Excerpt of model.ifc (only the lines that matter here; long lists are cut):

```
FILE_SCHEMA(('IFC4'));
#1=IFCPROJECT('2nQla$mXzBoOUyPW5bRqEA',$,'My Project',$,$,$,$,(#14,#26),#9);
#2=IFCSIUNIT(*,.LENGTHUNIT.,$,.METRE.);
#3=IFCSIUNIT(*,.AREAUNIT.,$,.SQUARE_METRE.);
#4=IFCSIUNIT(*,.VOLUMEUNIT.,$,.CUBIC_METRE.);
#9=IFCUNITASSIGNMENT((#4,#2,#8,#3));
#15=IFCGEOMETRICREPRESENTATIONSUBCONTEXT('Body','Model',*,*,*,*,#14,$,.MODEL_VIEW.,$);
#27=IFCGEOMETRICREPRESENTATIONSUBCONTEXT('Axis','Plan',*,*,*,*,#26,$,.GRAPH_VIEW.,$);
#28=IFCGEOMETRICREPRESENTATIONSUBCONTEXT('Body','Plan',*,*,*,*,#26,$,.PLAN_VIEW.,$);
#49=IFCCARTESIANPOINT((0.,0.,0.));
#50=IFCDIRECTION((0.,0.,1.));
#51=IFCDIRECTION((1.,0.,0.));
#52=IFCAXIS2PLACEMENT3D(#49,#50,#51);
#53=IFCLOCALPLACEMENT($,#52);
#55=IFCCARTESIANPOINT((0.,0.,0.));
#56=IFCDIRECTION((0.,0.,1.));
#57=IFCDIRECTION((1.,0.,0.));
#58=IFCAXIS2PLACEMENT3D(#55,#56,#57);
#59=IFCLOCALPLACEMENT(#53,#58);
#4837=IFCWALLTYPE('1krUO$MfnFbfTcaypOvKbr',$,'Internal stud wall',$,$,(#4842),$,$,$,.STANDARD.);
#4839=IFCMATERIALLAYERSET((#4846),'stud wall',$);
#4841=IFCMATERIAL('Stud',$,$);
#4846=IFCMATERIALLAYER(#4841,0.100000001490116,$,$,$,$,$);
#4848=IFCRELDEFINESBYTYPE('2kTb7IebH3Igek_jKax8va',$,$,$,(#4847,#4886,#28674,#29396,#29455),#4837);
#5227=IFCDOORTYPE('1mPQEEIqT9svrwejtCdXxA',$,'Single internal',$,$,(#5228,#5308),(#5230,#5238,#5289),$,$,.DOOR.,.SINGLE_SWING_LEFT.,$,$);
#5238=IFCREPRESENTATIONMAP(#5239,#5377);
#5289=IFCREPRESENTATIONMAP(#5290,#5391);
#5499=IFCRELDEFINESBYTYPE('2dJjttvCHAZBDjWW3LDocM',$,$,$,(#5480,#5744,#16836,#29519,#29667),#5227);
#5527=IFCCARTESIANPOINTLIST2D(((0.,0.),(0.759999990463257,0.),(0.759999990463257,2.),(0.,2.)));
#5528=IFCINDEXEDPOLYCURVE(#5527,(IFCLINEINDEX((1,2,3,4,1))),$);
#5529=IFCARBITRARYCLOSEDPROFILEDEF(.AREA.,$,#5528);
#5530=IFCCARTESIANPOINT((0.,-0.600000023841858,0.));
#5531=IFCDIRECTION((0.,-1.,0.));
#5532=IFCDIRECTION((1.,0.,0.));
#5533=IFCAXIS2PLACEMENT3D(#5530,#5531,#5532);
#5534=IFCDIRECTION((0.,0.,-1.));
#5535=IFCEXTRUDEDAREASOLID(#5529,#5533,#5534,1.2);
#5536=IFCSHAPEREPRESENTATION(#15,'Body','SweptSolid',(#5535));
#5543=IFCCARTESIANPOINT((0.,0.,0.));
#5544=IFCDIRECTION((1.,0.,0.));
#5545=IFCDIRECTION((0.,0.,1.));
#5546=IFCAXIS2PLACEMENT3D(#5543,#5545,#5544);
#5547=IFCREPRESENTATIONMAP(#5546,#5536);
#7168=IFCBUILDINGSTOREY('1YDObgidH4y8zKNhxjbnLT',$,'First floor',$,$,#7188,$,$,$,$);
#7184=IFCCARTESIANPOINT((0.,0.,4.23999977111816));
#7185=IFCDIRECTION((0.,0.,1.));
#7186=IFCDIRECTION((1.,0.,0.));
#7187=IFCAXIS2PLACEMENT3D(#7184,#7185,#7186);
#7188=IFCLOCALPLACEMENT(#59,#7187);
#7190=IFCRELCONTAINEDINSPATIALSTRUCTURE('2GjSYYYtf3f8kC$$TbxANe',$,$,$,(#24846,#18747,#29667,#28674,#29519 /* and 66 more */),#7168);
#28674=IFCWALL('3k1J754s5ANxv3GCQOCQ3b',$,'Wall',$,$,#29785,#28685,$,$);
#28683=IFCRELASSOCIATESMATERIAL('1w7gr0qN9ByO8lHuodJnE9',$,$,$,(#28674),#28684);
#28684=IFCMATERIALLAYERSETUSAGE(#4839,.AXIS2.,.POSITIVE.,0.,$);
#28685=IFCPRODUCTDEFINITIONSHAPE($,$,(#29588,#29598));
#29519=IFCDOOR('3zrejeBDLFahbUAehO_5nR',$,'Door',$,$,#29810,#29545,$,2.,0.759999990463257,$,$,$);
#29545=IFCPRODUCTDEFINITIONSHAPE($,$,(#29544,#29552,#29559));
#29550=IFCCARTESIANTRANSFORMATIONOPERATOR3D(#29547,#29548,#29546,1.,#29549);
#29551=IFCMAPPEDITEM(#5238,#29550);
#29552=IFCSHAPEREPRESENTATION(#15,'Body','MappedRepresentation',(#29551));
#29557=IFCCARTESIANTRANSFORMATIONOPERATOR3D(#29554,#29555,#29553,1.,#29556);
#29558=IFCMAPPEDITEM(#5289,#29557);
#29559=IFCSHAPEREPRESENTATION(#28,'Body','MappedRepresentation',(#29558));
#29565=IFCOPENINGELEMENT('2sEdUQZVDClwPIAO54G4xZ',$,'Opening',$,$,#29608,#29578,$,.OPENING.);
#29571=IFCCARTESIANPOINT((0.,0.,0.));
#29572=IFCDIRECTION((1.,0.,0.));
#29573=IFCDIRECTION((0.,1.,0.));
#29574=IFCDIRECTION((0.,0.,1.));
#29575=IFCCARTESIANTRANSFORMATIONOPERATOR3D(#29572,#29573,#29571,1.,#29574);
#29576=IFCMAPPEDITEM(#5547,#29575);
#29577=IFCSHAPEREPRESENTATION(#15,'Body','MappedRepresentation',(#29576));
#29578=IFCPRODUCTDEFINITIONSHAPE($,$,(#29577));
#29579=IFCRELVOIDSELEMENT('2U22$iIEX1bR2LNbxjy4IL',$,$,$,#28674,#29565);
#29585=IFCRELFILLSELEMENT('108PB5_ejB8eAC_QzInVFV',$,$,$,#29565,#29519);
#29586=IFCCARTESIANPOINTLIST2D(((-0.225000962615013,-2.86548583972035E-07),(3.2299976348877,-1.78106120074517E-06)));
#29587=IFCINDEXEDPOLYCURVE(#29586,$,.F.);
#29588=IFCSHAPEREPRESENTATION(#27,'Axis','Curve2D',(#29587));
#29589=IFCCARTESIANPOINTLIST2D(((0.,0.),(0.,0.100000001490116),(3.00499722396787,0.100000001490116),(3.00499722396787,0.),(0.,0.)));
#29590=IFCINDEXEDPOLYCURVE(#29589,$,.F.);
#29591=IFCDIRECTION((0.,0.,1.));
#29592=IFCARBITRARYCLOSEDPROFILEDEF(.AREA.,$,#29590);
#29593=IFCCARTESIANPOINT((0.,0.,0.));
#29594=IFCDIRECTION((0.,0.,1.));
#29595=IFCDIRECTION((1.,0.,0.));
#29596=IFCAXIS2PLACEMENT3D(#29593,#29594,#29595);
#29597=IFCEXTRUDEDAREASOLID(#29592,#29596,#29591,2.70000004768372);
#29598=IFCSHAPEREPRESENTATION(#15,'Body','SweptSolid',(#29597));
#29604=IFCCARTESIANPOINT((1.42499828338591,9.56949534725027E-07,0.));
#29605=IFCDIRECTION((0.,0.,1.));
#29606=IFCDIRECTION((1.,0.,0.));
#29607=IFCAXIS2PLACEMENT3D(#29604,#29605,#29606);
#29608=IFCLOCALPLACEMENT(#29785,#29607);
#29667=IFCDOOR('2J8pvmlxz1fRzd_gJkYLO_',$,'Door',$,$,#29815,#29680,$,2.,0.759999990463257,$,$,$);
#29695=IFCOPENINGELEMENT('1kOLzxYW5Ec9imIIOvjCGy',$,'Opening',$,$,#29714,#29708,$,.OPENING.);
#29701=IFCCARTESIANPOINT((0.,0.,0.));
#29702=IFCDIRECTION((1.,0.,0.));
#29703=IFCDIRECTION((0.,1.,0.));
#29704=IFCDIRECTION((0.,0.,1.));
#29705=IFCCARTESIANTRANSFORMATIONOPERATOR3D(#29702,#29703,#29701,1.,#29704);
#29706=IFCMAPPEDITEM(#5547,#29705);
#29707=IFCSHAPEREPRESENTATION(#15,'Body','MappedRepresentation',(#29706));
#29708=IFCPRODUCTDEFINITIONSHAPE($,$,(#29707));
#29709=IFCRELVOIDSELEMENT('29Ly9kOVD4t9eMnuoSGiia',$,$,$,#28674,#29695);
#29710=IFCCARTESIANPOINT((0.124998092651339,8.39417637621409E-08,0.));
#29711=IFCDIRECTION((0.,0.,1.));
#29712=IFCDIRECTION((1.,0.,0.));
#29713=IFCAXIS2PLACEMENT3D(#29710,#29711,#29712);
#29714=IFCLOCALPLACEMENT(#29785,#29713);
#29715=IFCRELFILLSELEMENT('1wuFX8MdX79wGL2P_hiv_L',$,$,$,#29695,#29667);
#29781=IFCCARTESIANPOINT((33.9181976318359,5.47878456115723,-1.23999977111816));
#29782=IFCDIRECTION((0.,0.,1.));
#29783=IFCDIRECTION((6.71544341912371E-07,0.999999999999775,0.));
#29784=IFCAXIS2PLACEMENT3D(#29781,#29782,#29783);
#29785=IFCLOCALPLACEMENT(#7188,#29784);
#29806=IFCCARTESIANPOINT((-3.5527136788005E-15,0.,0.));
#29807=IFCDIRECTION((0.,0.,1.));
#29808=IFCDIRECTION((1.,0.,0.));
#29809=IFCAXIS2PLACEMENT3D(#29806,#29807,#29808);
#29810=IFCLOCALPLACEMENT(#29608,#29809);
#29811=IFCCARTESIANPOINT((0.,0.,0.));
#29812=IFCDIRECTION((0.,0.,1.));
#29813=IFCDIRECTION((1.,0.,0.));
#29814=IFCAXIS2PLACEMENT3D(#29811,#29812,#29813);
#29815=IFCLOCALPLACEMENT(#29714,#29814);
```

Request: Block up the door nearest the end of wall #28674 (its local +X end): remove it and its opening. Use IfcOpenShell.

```python
import ifcopenshell
import ifcopenshell.api.feature
import ifcopenshell.api.root
import ifcopenshell.geom
import ifcopenshell.util.shape

model = ifcopenshell.open("model.ifc")
settings = ifcopenshell.geom.settings()


def volume(element):
    """Net volume in cubic metres, openings subtracted."""
    shape = ifcopenshell.geom.create_shape(settings, element)
    return ifcopenshell.util.shape.get_volume(shape.geometry)


door = model.by_id(29519)
opening = door.FillsVoids[0].RelatingOpeningElement
wall = opening.VoidsElements[0].RelatingBuildingElement
before = volume(wall)

ifcopenshell.api.root.remove_product(model, product=door)
ifcopenshell.api.feature.remove_feature(model, feature=opening)

after = volume(wall)

print(f"wall volume {before:.3f} -> {after:.3f} m3")

model.write("model-out.ifc")
```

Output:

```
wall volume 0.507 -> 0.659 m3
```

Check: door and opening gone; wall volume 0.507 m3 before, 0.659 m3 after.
